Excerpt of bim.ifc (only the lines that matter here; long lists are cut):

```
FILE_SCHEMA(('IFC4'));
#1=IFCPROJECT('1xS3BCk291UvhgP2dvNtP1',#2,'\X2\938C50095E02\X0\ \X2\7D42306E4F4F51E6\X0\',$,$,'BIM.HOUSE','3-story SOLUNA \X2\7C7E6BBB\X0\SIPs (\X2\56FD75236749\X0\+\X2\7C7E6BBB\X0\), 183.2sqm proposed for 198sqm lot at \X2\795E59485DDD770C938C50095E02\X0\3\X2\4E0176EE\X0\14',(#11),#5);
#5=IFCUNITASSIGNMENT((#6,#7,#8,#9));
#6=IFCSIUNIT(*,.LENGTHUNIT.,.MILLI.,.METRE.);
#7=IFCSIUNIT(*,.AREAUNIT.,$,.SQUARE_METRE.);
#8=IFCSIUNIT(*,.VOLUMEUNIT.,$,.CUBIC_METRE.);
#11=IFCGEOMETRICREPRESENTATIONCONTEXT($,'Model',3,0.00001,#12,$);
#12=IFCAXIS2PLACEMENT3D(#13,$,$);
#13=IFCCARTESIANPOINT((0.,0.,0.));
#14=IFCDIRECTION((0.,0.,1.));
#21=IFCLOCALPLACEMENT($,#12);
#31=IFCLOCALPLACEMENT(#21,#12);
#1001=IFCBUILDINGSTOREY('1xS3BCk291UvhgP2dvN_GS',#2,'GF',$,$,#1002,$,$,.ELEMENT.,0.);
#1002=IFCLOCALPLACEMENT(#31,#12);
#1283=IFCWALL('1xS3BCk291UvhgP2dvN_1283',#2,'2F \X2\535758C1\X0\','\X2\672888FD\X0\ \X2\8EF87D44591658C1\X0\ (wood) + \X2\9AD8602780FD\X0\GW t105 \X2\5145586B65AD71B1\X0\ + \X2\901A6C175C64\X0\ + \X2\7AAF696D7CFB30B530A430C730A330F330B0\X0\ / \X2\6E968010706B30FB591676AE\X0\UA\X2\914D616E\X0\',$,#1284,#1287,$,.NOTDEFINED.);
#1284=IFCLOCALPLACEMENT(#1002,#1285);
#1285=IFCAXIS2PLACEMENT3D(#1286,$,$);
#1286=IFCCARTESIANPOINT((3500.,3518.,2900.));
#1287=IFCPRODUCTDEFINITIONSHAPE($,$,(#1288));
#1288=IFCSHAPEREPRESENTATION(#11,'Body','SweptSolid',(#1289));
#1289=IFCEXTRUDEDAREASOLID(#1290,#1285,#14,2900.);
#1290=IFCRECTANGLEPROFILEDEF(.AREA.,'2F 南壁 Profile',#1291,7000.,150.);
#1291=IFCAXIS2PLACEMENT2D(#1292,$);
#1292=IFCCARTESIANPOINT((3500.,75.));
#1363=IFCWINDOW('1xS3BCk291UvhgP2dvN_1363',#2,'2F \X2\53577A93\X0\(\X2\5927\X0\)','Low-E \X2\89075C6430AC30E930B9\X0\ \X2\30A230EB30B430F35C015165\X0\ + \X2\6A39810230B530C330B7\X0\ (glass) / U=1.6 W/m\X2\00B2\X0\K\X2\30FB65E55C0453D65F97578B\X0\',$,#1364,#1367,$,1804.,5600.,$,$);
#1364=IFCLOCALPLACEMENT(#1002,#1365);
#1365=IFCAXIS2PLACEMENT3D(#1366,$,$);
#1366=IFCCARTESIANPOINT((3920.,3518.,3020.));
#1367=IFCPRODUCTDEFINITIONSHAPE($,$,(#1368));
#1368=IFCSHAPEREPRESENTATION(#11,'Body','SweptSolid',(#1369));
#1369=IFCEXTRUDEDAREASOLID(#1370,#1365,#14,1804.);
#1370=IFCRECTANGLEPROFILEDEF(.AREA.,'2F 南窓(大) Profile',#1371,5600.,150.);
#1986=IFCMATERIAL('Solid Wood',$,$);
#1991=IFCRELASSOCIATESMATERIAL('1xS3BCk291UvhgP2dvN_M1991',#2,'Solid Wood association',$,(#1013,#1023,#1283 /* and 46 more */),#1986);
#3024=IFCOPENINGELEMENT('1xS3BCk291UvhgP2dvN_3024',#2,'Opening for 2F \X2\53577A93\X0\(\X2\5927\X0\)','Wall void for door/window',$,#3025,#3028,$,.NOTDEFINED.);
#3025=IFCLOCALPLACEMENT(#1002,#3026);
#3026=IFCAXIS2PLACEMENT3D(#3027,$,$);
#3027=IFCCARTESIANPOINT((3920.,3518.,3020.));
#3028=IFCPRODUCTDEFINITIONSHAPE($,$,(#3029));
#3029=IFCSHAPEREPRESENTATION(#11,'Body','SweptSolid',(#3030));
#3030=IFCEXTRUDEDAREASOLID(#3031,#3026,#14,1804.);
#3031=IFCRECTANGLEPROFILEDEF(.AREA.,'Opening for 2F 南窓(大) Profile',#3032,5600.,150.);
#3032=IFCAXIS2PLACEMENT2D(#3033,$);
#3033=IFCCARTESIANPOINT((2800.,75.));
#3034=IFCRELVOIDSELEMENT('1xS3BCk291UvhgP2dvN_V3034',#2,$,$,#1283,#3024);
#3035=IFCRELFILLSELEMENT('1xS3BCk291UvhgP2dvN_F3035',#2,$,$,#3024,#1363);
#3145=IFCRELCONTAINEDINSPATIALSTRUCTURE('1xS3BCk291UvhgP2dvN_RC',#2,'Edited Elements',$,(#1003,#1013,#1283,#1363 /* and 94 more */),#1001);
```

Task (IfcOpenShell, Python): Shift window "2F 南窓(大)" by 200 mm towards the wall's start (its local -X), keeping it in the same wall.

```python
import ifcopenshell
import ifcopenshell.api.geometry
import ifcopenshell.util.placement

model = ifcopenshell.open("bim.ifc")

window = model.by_id(1363)
opening = window.FillsVoids[0].RelatingOpeningElement
wall = opening.VoidsElements[0].RelatingBuildingElement

wall_matrix = ifcopenshell.util.placement.get_local_placement(wall.ObjectPlacement)
shift = wall_matrix[:3, 0] * -200.0
before = ifcopenshell.util.placement.get_local_placement(window.ObjectPlacement)[:3, 3].copy()

# The window is not placed relative to its opening, so move both.
for product in (opening, window):
    matrix = ifcopenshell.util.placement.get_local_placement(product.ObjectPlacement)
    matrix[:3, 3] += shift
    ifcopenshell.api.geometry.edit_object_placement(model, product=product, matrix=matrix, is_si=False)

after = ifcopenshell.util.placement.get_local_placement(window.ObjectPlacement)[:3, 3]
print("window moved by", (after - before).round(3) + 0.0)

model.write("bim_rev.ifc")
```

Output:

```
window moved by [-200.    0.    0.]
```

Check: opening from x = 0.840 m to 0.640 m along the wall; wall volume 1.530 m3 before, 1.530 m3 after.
